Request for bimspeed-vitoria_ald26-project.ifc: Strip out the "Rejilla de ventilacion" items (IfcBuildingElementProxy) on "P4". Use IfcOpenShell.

First a look at what the model holds.

```python
import ifcopenshell
import ifcopenshell.util.element

model = ifcopenshell.open("bimspeed-vitoria_ald26-project.ifc")
print(model.schema)
storey = next(s for s in model.by_type("IfcBuildingStorey") if s.Name == "P4")
proxies = [e for e in ifcopenshell.util.element.get_decomposition(storey) if e.is_a("IfcBuildingElementProxy")]
seen = {}
for e in proxies:
    element_type = ifcopenshell.util.element.get_type(e)
    name = element_type.Name if element_type not in (None, e) else None
    seen[name] = seen.get(name, 0) + 1
for name, count in sorted(seen.items(), key=str):
    print(count, "x", name)
```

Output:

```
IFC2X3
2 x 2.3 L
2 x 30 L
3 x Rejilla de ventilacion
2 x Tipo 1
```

```python
import ifcopenshell
import ifcopenshell.api.root
import ifcopenshell.util.element

model = ifcopenshell.open("bimspeed-vitoria_ald26-project.ifc")

storey = next(s for s in model.by_type("IfcBuildingStorey") if s.Name == "P4")
proxies = [e for e in ifcopenshell.util.element.get_decomposition(storey) if e.is_a("IfcBuildingElementProxy")]
targets = [e for e in proxies if (t := ifcopenshell.util.element.get_type(e)) not in (None, e) and t.Name == "Rejilla de ventilacion"]

for e in targets:
    ifcopenshell.api.root.remove_product(model, product=e)
print(len(targets), "removed")

model.write("bimspeed-vitoria_ald26-project-out.ifc")
```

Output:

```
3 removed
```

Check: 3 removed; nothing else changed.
